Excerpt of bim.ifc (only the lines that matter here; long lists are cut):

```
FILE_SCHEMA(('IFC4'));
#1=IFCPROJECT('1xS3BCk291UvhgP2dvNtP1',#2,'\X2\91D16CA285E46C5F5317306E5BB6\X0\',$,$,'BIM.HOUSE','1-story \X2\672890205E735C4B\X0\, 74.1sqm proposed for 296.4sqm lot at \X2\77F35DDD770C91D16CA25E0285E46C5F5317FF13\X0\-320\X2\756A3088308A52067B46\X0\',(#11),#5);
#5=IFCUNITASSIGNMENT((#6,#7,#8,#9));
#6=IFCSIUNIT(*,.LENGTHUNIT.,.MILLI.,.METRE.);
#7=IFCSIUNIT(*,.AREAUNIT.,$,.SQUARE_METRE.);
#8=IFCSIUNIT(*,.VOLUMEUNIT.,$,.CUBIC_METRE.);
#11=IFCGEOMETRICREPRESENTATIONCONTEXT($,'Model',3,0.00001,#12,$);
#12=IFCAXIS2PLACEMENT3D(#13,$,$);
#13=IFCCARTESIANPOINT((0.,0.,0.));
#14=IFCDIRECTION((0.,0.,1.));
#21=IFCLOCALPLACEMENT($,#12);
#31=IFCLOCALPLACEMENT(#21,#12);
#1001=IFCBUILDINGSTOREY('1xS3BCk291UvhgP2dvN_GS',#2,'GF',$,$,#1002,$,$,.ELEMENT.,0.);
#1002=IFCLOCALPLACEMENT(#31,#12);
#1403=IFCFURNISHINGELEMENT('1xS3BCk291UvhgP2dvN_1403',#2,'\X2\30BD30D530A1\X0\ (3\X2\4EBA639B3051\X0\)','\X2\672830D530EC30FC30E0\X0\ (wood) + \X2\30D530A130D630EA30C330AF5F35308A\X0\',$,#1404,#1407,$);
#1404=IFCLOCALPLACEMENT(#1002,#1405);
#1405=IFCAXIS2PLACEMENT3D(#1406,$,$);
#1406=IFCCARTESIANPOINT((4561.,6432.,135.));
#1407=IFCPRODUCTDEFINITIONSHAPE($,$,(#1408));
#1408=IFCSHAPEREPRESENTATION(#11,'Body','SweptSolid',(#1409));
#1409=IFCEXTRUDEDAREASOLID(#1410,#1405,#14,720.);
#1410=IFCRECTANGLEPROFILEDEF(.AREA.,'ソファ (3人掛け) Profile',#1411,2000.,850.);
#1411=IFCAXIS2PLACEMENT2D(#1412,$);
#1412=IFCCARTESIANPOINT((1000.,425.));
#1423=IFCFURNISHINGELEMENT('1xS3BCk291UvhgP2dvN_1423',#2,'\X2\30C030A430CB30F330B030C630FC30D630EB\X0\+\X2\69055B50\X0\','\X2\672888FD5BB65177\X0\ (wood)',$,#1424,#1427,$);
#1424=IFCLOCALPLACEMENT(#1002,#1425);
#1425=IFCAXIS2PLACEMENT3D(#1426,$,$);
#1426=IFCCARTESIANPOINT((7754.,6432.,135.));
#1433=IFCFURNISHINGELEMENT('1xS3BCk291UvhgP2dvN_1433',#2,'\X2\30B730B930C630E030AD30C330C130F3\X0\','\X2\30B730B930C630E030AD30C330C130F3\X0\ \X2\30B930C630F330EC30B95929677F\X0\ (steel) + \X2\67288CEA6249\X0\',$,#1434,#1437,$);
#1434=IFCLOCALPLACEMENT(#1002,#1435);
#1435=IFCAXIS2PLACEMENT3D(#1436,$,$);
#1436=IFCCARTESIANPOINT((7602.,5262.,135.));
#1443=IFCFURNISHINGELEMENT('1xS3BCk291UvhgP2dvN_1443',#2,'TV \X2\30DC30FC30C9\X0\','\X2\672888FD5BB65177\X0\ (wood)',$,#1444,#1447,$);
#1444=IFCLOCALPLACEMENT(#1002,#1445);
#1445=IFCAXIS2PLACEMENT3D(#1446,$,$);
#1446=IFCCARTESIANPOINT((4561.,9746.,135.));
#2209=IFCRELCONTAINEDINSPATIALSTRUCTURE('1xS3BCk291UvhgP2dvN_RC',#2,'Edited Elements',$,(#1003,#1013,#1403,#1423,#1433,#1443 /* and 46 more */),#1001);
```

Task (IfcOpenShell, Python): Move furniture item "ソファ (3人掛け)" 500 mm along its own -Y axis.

```python
import ifcopenshell
import ifcopenshell.api.geometry
import ifcopenshell.util.placement

model = ifcopenshell.open("bim.ifc")

item = model.by_id(1403)
matrix = ifcopenshell.util.placement.get_local_placement(item.ObjectPlacement)
matrix[:3, 3] -= matrix[:3, 1] * 500.0
ifcopenshell.api.geometry.edit_object_placement(model, product=item, matrix=matrix, is_si=False)

print(ifcopenshell.util.placement.get_local_placement(item.ObjectPlacement).round(3) + 0.0)

model.write("bim-out.ifc")
```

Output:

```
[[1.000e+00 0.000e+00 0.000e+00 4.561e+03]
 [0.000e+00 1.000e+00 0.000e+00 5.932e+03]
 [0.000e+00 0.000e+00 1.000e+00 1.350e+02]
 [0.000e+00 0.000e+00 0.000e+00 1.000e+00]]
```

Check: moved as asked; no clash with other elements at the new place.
